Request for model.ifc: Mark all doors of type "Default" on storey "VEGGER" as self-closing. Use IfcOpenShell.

First a look at what the model holds.

```python
import ifcopenshell
import ifcopenshell.util.element

model = ifcopenshell.open("model.ifc")
print(model.schema)
storey = next(s for s in model.by_type("IfcBuildingStorey") if s.Name == "VEGGER")
doors = [e for e in ifcopenshell.util.element.get_decomposition(storey) if e.is_a("IfcDoor")]
seen = {}
for e in doors:
    element_type = ifcopenshell.util.element.get_type(e)
    key = (element_type.Name if element_type != e and element_type else None, ifcopenshell.util.element.get_pset(e, "Pset_DoorCommon", "SelfClosing"))
    seen[key] = seen.get(key, 0) + 1
for (name, value), count in sorted(seen.items(), key=str):
    print(count, "x", name, "|", value)
```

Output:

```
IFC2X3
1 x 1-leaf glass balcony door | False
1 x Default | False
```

```python
import ifcopenshell
import ifcopenshell.api.pset
import ifcopenshell.util.element

model = ifcopenshell.open("model.ifc")

storey = next(s for s in model.by_type("IfcBuildingStorey") if s.Name == "VEGGER")
doors = [e for e in ifcopenshell.util.element.get_decomposition(storey) if e.is_a("IfcDoor")]

count = 0
for e in doors:
    element_type = ifcopenshell.util.element.get_type(e)
    if element_type in (None, e) or element_type.Name != "Default":
        continue
    # add_pset returns the element's existing set when there is one.
    pset = ifcopenshell.api.pset.add_pset(model, product=e, name="Pset_DoorCommon")
    ifcopenshell.api.pset.edit_pset(model, pset=pset, properties={"SelfClosing": True})
    count += 1

print(count, "doors updated")

model.write("model-out.ifc")
```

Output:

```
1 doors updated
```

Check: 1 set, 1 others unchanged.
